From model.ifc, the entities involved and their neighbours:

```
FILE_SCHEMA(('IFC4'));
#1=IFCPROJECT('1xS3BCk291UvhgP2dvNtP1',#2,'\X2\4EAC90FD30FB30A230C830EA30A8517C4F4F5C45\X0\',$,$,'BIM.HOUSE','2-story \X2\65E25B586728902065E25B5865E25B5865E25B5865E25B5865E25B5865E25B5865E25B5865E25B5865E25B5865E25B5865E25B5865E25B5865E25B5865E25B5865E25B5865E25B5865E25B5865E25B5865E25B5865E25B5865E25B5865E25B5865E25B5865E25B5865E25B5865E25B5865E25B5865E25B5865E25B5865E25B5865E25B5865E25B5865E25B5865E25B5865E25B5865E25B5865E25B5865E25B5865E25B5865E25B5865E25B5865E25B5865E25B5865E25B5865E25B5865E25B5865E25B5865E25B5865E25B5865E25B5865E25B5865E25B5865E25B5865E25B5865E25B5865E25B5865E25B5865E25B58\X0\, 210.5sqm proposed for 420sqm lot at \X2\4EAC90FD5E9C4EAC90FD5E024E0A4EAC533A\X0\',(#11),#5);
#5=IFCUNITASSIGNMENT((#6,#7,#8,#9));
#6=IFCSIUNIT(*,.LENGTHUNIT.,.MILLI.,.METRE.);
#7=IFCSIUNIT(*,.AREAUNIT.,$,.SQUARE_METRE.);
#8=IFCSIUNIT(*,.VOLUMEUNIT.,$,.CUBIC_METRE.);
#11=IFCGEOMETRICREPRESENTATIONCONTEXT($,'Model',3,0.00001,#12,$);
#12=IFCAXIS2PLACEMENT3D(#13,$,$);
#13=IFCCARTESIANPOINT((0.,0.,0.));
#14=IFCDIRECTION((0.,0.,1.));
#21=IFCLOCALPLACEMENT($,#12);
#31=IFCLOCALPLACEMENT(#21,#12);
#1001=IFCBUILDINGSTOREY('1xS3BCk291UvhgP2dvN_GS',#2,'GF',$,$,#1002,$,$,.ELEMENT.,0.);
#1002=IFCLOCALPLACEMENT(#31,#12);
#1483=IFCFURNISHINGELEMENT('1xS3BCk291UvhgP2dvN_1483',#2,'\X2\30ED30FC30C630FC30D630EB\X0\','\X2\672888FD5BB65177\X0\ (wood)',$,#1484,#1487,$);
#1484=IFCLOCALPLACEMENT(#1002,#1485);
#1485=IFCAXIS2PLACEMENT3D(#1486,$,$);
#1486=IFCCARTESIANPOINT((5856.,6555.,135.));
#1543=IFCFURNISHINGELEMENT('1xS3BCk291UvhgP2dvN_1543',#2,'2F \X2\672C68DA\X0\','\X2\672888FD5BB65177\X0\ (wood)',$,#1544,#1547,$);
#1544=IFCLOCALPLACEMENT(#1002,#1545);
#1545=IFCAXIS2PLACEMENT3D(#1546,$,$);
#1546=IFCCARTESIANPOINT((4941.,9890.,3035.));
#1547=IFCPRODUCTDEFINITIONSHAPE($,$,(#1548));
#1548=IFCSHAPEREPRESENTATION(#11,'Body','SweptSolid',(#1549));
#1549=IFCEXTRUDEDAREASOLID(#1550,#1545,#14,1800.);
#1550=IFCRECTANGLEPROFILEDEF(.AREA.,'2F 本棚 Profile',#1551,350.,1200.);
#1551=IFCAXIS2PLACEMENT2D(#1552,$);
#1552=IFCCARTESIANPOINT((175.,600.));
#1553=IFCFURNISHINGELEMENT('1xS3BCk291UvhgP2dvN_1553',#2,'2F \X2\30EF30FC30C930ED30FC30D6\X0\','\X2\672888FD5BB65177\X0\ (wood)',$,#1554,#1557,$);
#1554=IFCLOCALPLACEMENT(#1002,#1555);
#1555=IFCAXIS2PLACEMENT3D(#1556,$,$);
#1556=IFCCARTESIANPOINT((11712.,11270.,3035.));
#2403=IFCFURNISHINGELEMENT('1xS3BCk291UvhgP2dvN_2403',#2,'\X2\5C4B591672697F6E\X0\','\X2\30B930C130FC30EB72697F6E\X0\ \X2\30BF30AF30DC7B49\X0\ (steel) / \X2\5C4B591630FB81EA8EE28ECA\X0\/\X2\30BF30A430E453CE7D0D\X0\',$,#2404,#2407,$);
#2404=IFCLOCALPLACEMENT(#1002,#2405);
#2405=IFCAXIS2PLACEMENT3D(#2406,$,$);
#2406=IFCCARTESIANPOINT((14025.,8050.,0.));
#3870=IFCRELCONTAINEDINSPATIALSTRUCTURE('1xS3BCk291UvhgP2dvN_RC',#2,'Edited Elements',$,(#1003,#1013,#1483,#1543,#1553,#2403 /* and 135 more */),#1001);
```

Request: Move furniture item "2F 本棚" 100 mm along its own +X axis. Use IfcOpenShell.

```python
import ifcopenshell
import ifcopenshell.api.geometry
import ifcopenshell.util.placement

model = ifcopenshell.open("model.ifc")

item = model.by_guid("1xS3BCk291UvhgP2dvN_1543")
matrix = ifcopenshell.util.placement.get_local_placement(item.ObjectPlacement)
matrix[:3, 3] += matrix[:3, 0] * 100.0
ifcopenshell.api.geometry.edit_object_placement(model, product=item, matrix=matrix, is_si=False)

print(ifcopenshell.util.placement.get_local_placement(item.ObjectPlacement).round(3) + 0.0)

model.write("model_edited.ifc")
```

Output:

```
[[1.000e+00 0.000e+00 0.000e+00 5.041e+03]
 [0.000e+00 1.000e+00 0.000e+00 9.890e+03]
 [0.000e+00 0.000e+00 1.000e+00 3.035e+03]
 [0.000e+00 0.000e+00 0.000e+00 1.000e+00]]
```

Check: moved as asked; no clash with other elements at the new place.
